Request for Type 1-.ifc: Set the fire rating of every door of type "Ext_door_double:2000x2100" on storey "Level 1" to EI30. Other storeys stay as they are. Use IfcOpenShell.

First a look at what the model holds.

```python
import ifcopenshell
import ifcopenshell.util.element

model = ifcopenshell.open("Type 1-.ifc")
print(model.schema)
storey = next(s for s in model.by_type("IfcBuildingStorey") if s.Name == "Level 1")
doors = [e for e in ifcopenshell.util.element.get_decomposition(storey) if e.is_a("IfcDoor")]
seen = {}
for e in doors:
    element_type = ifcopenshell.util.element.get_type(e)
    key = (element_type.Name if element_type != e and element_type else None, ifcopenshell.util.element.get_pset(e, "Pset_DoorCommon", "FireRating"))
    seen[key] = seen.get(key, 0) + 1
for (name, value), count in sorted(seen.items(), key=str):
    print(count, "x", name, "|", value)
```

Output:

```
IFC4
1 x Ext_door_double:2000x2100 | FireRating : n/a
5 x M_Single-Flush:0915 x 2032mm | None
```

```python
import ifcopenshell
import ifcopenshell.api.pset
import ifcopenshell.util.element

model = ifcopenshell.open("Type 1-.ifc")

storey = next(s for s in model.by_type("IfcBuildingStorey") if s.Name == "Level 1")
doors = [e for e in ifcopenshell.util.element.get_decomposition(storey) if e.is_a("IfcDoor")]

count = 0
for e in doors:
    element_type = ifcopenshell.util.element.get_type(e)
    if element_type in (None, e) or element_type.Name != "Ext_door_double:2000x2100":
        continue
    # add_pset returns the element's existing set when there is one.
    pset = ifcopenshell.api.pset.add_pset(model, product=e, name="Pset_DoorCommon")
    ifcopenshell.api.pset.edit_pset(model, pset=pset, properties={"FireRating": "EI30"})
    count += 1

print(count, "doors updated")

model.write("Type 1-_edited.ifc")
```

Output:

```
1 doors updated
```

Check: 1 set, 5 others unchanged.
